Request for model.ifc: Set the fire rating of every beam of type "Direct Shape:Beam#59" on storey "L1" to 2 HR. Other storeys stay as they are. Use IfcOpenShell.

First a look at what the model holds.

```python
import ifcopenshell
import ifcopenshell.util.element

model = ifcopenshell.open("model.ifc")
print(model.schema)
storey = next(s for s in model.by_type("IfcBuildingStorey") if s.Name == "L1")
beams = [e for e in ifcopenshell.util.element.get_decomposition(storey) if e.is_a("IfcBeam")]
seen = {}
for e in beams:
    element_type = ifcopenshell.util.element.get_type(e)
    key = (element_type.Name if element_type != e and element_type else None, ifcopenshell.util.element.get_pset(e, "Pset_BeamCommon", "FireRating"))
    seen[key] = seen.get(key, 0) + 1
for (name, value), count in sorted(seen.items(), key=str):
    print(count, "x", name, "|", value)
```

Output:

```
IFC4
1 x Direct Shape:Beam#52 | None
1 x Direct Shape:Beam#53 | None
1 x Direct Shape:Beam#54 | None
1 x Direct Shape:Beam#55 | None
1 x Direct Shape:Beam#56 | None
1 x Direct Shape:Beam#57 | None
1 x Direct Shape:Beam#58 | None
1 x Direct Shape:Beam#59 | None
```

```python
import ifcopenshell
import ifcopenshell.api.pset
import ifcopenshell.util.element

model = ifcopenshell.open("model.ifc")

storey = next(s for s in model.by_type("IfcBuildingStorey") if s.Name == "L1")
beams = [e for e in ifcopenshell.util.element.get_decomposition(storey) if e.is_a("IfcBeam")]

count = 0
for e in beams:
    element_type = ifcopenshell.util.element.get_type(e)
    if element_type in (None, e) or element_type.Name != "Direct Shape:Beam#59":
        continue
    # add_pset returns the element's existing set when there is one.
    pset = ifcopenshell.api.pset.add_pset(model, product=e, name="Pset_BeamCommon")
    ifcopenshell.api.pset.edit_pset(model, pset=pset, properties={"FireRating": "2 HR"})
    count += 1

print(count, "beams updated")

model.write("model_rev.ifc")
```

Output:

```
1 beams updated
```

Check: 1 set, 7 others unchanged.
